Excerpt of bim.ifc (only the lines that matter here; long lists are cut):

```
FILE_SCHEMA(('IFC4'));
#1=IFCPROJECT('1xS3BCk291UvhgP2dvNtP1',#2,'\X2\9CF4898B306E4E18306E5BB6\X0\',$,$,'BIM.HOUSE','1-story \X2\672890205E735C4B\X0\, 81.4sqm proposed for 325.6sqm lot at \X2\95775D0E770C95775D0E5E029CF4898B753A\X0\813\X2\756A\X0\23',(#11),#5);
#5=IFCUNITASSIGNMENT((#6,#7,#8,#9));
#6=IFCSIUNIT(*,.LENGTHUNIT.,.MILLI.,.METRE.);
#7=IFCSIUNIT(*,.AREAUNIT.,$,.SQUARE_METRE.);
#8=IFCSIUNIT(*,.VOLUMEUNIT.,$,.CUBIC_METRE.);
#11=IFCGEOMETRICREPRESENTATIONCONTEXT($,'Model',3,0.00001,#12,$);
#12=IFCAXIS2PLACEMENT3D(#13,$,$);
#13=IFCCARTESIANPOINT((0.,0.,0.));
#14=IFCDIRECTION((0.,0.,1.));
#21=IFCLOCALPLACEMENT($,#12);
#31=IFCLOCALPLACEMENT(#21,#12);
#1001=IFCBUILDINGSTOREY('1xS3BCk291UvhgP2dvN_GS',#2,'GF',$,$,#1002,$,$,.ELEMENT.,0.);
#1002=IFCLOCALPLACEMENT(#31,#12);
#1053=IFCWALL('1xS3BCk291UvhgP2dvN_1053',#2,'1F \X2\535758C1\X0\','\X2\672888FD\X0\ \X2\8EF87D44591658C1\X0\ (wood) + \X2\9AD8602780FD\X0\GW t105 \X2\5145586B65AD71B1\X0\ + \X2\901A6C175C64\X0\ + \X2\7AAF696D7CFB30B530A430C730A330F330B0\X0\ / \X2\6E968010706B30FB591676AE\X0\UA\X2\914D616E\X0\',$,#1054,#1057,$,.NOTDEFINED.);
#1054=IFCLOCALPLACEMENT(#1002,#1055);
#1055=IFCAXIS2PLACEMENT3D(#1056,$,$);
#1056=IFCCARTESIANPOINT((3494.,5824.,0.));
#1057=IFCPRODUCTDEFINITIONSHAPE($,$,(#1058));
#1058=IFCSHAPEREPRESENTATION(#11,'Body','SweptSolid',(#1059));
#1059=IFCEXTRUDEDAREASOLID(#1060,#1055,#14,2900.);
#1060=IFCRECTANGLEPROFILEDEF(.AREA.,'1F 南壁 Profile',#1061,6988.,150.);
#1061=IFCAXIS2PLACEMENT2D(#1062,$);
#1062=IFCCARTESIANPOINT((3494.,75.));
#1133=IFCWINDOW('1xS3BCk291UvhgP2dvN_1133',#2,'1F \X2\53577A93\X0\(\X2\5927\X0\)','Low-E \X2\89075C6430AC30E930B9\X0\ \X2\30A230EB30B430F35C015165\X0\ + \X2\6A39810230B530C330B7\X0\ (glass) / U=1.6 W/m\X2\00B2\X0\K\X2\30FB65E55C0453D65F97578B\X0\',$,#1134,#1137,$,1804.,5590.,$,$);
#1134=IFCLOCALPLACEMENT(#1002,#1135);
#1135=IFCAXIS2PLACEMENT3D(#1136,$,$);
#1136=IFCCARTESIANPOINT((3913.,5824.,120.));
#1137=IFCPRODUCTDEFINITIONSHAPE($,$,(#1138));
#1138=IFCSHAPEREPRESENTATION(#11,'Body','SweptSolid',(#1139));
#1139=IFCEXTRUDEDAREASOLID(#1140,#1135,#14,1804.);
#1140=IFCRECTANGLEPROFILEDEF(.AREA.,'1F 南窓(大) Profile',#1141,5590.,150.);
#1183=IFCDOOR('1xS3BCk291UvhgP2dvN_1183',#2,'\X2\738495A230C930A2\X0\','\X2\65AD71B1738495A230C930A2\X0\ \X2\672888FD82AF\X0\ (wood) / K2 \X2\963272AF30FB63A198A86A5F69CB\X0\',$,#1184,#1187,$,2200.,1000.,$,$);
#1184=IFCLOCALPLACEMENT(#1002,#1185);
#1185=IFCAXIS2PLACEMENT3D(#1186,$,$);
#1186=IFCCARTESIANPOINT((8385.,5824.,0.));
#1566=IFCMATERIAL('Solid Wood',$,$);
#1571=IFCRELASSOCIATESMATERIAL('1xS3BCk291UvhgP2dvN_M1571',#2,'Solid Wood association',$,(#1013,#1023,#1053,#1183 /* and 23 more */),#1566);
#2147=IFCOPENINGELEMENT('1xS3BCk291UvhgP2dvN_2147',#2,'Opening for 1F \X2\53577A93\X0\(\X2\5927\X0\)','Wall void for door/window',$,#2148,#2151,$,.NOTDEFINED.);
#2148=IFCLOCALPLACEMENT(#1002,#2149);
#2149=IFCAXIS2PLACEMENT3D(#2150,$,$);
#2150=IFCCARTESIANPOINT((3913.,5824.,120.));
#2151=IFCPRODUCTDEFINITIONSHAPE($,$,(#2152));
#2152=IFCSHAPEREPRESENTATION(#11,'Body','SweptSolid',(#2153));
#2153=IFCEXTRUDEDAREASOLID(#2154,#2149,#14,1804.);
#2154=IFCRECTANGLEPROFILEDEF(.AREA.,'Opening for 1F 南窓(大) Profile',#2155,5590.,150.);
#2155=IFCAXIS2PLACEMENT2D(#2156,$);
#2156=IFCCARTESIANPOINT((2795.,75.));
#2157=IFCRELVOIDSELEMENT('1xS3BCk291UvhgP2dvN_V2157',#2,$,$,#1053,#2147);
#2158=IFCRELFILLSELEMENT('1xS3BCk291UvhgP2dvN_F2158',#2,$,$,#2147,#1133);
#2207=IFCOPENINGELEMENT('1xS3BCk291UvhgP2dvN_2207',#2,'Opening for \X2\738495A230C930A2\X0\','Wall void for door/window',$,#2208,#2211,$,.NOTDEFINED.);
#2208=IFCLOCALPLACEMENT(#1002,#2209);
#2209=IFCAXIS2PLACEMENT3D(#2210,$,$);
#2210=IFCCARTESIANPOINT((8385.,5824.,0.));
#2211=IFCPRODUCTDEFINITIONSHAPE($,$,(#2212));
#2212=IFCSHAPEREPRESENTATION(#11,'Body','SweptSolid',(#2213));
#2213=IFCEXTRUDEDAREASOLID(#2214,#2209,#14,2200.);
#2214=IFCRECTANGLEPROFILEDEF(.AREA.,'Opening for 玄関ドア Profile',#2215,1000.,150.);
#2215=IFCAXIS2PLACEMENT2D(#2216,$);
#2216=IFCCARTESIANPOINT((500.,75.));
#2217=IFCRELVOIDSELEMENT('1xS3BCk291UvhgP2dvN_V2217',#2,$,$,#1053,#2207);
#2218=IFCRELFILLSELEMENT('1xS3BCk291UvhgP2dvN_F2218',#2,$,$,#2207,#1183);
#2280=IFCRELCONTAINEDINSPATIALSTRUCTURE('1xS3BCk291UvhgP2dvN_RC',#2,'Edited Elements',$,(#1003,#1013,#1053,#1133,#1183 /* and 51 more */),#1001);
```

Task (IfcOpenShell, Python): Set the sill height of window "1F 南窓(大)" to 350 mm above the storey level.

```python
import numpy as np
import ifcopenshell
import ifcopenshell.api.geometry
import ifcopenshell.geom
import ifcopenshell.util.element
import ifcopenshell.util.placement
import ifcopenshell.util.shape
import ifcopenshell.util.unit

model = ifcopenshell.open("bim.ifc")
unit_scale = ifcopenshell.util.unit.calculate_unit_scale(model)

window = model.by_id(1133)
opening = window.FillsVoids[0].RelatingOpeningElement
storey = ifcopenshell.util.element.get_container(window, ifc_class="IfcBuildingStorey")
level = ifcopenshell.util.placement.get_local_placement(storey.ObjectPlacement)[2, 3]

# The opening's origin need not be at the sill, so measure its lowest point.
shape = ifcopenshell.geom.create_shape(ifcopenshell.geom.settings(), opening)
bottom = ifcopenshell.util.shape.get_shape_bottom_elevation(shape, shape.geometry) / unit_scale
dz = level + 350.0 - bottom

shift = np.array([0.0, 0.0, dz])
# The window is not placed relative to its opening, so move both.
for product in (opening, window):
    matrix = ifcopenshell.util.placement.get_local_placement(product.ObjectPlacement)
    matrix[:3, 3] += shift
    ifcopenshell.api.geometry.edit_object_placement(model, product=product, matrix=matrix, is_si=False)

print(f"moved by {dz * unit_scale:+.3f} m")

model.write("bim_rev.ifc")
```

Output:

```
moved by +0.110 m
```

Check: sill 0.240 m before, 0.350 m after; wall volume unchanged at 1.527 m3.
